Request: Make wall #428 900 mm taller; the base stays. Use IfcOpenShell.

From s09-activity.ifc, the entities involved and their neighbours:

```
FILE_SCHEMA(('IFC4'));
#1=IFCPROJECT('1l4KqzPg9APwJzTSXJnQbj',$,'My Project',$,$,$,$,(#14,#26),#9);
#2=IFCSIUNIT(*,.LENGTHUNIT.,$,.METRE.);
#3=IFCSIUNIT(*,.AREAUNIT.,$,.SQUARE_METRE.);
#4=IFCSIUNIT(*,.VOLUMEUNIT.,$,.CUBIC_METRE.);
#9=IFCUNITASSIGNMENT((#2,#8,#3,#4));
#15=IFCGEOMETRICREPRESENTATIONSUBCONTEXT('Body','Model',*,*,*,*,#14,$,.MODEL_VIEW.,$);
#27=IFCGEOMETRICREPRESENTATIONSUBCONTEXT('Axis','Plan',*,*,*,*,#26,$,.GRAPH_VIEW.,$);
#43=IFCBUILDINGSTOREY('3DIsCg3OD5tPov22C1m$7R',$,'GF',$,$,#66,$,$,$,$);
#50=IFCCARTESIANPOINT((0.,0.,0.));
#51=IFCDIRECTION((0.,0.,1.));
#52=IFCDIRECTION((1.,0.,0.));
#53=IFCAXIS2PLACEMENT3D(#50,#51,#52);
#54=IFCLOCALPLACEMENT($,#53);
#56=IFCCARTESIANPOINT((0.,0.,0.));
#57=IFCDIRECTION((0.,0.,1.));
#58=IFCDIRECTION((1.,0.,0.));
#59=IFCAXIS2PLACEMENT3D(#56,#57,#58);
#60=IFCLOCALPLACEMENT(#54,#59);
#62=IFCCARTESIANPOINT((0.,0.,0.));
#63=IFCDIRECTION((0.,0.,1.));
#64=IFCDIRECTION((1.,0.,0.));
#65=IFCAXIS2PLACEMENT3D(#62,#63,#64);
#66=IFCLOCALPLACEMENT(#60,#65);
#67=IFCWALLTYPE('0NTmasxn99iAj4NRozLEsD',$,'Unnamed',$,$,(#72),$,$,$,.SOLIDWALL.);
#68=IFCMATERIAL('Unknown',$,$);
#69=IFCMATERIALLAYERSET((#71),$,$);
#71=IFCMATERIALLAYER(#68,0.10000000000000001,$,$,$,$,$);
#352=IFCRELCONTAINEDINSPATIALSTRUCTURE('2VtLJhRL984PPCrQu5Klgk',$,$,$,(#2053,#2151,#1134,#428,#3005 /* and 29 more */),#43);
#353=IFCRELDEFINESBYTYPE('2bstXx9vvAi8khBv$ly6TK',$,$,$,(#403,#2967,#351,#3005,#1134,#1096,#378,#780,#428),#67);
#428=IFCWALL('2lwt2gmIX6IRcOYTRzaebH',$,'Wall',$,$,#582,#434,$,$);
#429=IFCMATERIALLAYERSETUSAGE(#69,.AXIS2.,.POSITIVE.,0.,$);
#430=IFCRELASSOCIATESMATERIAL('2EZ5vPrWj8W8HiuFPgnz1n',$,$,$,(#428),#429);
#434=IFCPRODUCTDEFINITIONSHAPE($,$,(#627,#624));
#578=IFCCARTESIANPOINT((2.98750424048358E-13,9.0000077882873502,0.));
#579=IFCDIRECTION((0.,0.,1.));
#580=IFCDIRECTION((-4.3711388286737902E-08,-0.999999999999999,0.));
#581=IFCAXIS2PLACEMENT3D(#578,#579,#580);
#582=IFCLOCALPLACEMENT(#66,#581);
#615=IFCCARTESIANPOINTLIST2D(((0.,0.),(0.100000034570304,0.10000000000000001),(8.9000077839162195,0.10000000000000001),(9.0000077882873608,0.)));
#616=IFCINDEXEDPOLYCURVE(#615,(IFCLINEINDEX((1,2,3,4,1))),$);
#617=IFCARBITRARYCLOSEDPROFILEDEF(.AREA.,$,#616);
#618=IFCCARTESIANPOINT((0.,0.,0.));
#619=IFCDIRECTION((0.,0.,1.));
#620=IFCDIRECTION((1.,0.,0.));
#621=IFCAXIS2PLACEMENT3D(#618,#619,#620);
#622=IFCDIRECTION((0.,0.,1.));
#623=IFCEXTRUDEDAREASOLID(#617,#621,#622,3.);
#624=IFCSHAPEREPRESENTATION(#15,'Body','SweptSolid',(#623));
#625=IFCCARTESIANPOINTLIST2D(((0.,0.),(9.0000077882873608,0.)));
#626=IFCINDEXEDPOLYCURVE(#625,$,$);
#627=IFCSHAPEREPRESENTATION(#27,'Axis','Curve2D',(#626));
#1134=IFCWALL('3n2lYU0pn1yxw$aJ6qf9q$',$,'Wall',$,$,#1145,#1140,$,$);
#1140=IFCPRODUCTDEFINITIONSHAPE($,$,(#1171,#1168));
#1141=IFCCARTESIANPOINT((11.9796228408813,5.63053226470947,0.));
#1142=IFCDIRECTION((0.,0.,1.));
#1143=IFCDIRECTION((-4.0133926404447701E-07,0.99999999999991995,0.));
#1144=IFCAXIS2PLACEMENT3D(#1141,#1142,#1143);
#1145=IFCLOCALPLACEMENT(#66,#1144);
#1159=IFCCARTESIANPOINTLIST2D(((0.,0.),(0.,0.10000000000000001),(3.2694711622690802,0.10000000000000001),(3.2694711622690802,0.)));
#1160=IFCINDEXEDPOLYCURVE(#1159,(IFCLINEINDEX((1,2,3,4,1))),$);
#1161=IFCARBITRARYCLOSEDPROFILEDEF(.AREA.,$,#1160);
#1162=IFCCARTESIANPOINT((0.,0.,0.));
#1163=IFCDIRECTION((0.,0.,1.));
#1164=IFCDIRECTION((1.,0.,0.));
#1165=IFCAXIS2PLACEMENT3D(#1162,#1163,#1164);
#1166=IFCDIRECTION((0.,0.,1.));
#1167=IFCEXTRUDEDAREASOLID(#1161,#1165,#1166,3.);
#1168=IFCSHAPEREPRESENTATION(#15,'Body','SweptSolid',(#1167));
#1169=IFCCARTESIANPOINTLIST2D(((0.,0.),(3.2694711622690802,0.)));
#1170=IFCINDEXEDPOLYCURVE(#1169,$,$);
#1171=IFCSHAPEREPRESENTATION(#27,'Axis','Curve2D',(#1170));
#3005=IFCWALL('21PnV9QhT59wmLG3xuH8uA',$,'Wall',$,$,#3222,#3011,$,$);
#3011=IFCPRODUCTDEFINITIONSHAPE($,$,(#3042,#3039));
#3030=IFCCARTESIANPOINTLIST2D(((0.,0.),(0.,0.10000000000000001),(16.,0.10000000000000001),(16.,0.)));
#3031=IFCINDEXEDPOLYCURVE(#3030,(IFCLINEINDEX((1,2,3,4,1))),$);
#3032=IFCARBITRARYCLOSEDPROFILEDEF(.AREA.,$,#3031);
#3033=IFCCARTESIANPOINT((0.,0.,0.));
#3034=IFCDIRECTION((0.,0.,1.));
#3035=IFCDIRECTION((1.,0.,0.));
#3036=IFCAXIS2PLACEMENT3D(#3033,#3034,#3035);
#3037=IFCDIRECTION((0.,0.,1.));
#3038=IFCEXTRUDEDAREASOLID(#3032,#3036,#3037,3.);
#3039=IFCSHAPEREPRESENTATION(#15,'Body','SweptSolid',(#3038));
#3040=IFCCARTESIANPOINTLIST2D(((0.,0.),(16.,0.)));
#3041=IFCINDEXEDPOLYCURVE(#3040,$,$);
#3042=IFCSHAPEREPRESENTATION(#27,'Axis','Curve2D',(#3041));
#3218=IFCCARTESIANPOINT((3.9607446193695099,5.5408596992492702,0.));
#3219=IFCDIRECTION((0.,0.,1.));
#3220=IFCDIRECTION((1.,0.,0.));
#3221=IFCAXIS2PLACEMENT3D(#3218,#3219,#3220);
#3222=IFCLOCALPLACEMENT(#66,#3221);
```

```python
import ifcopenshell
import ifcopenshell.geom
import ifcopenshell.util.representation
import ifcopenshell.util.shape

model = ifcopenshell.open("s09-activity.ifc")
settings = ifcopenshell.geom.settings()


def volume(element):
    """Net volume in cubic metres, openings subtracted."""
    shape = ifcopenshell.geom.create_shape(settings, element)
    return ifcopenshell.util.shape.get_volume(shape.geometry)


wall = model.by_id(428)
before = volume(wall)

body = ifcopenshell.util.representation.get_representation(wall, "Model", "Body")
solid = body.Items[0]
old_height = solid.Depth
solid.Depth += 0.9
after = volume(wall)

print(f"height {old_height:g} -> {solid.Depth:g}, volume {before:.3f} -> {after:.3f} m3")

model.write("s09-activity_updated.ifc")
```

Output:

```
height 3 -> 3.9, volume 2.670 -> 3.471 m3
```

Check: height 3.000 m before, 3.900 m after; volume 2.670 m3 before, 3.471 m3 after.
